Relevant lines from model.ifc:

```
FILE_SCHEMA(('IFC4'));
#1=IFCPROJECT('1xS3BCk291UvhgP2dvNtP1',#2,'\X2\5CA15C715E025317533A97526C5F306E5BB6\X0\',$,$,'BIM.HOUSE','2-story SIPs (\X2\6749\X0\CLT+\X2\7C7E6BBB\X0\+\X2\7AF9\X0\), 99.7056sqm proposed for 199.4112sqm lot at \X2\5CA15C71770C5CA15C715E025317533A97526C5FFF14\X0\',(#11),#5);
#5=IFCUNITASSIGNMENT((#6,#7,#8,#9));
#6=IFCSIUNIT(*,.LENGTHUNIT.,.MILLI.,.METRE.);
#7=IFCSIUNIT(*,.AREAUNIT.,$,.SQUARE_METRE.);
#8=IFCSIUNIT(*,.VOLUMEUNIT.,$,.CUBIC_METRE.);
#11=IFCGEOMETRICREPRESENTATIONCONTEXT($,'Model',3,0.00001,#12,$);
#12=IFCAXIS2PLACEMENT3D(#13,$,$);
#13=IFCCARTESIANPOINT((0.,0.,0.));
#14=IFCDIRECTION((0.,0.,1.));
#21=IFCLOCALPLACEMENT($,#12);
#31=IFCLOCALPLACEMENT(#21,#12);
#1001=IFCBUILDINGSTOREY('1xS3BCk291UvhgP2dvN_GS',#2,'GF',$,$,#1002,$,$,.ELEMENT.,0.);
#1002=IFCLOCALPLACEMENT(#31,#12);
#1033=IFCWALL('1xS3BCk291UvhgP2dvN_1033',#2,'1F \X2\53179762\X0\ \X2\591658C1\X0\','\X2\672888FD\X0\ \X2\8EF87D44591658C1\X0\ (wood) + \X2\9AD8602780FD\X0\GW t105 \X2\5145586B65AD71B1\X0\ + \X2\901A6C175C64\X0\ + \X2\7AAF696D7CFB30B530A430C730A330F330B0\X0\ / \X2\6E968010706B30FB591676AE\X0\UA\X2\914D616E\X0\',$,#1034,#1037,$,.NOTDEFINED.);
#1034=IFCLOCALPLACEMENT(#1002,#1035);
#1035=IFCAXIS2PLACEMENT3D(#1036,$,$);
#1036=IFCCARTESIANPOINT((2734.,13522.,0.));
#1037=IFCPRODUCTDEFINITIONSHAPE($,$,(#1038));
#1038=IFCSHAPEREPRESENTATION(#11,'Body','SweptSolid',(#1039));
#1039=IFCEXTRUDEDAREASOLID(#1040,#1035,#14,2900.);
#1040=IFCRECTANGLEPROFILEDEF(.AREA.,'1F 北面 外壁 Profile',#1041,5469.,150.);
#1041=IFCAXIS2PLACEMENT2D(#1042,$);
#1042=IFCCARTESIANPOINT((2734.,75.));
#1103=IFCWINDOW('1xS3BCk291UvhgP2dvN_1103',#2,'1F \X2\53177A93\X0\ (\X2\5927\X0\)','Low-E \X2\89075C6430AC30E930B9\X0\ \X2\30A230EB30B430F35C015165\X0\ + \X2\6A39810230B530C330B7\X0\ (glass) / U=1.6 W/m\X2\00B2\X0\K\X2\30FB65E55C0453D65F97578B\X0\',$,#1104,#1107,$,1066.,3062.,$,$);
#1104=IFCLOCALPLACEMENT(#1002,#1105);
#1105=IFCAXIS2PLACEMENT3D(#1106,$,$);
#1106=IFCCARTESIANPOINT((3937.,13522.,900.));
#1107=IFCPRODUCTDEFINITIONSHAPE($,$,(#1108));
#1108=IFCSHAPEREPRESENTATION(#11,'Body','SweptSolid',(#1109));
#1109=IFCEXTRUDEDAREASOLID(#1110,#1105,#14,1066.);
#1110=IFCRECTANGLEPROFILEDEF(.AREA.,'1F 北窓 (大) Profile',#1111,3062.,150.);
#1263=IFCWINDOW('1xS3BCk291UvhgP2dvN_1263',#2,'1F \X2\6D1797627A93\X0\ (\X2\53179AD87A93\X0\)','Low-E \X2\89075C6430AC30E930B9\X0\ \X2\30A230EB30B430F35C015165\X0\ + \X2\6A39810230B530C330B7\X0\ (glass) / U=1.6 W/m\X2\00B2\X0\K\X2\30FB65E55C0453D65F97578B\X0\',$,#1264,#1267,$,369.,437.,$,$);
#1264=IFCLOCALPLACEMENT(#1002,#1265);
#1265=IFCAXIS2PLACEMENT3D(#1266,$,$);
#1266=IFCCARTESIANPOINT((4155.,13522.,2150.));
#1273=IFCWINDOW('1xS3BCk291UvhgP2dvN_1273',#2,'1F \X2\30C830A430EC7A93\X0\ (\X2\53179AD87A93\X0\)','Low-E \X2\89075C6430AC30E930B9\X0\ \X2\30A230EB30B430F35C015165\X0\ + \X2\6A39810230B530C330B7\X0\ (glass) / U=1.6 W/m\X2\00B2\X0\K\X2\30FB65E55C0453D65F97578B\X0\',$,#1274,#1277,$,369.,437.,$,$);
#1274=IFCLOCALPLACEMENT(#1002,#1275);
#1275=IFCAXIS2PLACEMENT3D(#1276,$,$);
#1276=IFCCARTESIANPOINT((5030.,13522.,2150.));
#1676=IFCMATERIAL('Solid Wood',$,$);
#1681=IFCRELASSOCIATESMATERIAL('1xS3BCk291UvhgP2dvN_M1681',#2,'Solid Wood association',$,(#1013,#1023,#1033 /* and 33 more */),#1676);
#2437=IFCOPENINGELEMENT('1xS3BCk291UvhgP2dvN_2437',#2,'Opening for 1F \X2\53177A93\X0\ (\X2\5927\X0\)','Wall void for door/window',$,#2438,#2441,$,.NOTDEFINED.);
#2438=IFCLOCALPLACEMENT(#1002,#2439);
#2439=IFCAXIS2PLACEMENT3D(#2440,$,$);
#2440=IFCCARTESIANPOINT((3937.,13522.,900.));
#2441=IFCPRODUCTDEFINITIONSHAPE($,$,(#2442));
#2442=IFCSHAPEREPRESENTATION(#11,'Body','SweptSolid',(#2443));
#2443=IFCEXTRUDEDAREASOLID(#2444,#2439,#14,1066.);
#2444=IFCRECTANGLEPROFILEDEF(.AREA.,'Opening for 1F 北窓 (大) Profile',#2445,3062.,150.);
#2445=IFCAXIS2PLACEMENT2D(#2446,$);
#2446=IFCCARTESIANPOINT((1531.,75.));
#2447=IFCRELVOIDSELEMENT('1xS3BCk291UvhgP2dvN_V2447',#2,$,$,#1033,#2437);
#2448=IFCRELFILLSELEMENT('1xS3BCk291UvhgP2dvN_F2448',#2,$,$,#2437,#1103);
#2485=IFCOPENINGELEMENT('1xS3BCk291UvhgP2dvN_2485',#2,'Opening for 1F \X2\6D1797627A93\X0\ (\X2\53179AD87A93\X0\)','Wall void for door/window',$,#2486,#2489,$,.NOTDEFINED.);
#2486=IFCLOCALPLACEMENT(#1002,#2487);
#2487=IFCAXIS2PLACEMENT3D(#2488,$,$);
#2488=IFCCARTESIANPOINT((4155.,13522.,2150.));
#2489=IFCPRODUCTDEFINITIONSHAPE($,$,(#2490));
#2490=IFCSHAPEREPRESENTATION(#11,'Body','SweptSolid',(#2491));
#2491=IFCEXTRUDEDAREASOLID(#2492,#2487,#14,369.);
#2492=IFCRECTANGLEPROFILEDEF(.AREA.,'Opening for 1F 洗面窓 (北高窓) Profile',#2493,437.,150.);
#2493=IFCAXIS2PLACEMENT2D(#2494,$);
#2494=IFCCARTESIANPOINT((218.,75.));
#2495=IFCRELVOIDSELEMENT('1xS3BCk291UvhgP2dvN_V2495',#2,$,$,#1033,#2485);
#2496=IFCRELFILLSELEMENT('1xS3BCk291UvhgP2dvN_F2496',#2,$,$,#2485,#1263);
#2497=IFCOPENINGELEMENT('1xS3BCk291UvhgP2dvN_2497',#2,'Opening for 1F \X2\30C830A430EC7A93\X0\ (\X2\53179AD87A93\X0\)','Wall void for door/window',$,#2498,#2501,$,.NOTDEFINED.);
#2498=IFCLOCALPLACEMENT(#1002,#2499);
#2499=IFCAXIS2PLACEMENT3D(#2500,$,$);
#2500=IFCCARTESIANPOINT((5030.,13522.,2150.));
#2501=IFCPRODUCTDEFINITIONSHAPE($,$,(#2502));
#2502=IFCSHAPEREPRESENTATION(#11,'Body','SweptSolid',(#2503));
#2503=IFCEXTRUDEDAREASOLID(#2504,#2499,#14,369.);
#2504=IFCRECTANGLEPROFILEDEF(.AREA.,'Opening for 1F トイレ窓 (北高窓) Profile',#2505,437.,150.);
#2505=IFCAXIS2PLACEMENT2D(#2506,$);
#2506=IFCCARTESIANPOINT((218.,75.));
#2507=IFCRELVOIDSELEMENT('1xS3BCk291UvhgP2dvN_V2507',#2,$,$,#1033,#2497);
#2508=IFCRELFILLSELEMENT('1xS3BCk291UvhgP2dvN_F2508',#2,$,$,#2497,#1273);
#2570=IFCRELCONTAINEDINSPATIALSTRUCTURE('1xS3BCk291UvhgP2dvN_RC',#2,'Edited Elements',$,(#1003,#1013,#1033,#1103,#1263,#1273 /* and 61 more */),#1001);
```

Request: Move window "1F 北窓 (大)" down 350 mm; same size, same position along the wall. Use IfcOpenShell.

```python
import numpy as np
import ifcopenshell
import ifcopenshell.api.geometry
import ifcopenshell.util.placement
import ifcopenshell.util.unit

model = ifcopenshell.open("model.ifc")
unit_scale = ifcopenshell.util.unit.calculate_unit_scale(model)

window = model.by_guid("1xS3BCk291UvhgP2dvN_1103")
opening = window.FillsVoids[0].RelatingOpeningElement
dz = -0.35 / unit_scale

shift = np.array([0.0, 0.0, dz])
# The window is not placed relative to its opening, so move both.
for product in (opening, window):
    matrix = ifcopenshell.util.placement.get_local_placement(product.ObjectPlacement)
    matrix[:3, 3] += shift
    ifcopenshell.api.geometry.edit_object_placement(model, product=product, matrix=matrix, is_si=False)

print(f"moved by {dz * unit_scale:+.3f} m")

model.write("model-out.ifc")
```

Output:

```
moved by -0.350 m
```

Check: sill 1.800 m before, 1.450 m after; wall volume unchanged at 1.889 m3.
